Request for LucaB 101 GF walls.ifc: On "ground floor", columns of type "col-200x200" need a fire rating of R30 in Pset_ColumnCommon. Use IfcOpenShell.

First a look at what the model holds.

```python
import ifcopenshell
import ifcopenshell.util.element

model = ifcopenshell.open("LucaB 101 GF walls.ifc")
print(model.schema)
storey = next(s for s in model.by_type("IfcBuildingStorey") if s.Name == "ground floor")
columns = [e for e in ifcopenshell.util.element.get_decomposition(storey) if e.is_a("IfcColumn")]
seen = {}
for e in columns:
    element_type = ifcopenshell.util.element.get_type(e)
    key = (element_type.Name if element_type != e and element_type else None, ifcopenshell.util.element.get_pset(e, "Pset_ColumnCommon", "FireRating"))
    seen[key] = seen.get(key, 0) + 1
for (name, value), count in sorted(seen.items(), key=str):
    print(count, "x", name, "|", value)
```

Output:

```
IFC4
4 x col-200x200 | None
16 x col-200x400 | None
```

```python
import ifcopenshell
import ifcopenshell.api.pset
import ifcopenshell.util.element

model = ifcopenshell.open("LucaB 101 GF walls.ifc")

storey = next(s for s in model.by_type("IfcBuildingStorey") if s.Name == "ground floor")
columns = [e for e in ifcopenshell.util.element.get_decomposition(storey) if e.is_a("IfcColumn")]

count = 0
for e in columns:
    element_type = ifcopenshell.util.element.get_type(e)
    if element_type in (None, e) or element_type.Name != "col-200x200":
        continue
    # add_pset returns the element's existing set when there is one.
    pset = ifcopenshell.api.pset.add_pset(model, product=e, name="Pset_ColumnCommon")
    ifcopenshell.api.pset.edit_pset(model, pset=pset, properties={"FireRating": "R30"})
    count += 1

print(count, "columns updated")

model.write("LucaB 101 GF walls_edited.ifc")
```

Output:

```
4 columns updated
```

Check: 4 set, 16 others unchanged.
